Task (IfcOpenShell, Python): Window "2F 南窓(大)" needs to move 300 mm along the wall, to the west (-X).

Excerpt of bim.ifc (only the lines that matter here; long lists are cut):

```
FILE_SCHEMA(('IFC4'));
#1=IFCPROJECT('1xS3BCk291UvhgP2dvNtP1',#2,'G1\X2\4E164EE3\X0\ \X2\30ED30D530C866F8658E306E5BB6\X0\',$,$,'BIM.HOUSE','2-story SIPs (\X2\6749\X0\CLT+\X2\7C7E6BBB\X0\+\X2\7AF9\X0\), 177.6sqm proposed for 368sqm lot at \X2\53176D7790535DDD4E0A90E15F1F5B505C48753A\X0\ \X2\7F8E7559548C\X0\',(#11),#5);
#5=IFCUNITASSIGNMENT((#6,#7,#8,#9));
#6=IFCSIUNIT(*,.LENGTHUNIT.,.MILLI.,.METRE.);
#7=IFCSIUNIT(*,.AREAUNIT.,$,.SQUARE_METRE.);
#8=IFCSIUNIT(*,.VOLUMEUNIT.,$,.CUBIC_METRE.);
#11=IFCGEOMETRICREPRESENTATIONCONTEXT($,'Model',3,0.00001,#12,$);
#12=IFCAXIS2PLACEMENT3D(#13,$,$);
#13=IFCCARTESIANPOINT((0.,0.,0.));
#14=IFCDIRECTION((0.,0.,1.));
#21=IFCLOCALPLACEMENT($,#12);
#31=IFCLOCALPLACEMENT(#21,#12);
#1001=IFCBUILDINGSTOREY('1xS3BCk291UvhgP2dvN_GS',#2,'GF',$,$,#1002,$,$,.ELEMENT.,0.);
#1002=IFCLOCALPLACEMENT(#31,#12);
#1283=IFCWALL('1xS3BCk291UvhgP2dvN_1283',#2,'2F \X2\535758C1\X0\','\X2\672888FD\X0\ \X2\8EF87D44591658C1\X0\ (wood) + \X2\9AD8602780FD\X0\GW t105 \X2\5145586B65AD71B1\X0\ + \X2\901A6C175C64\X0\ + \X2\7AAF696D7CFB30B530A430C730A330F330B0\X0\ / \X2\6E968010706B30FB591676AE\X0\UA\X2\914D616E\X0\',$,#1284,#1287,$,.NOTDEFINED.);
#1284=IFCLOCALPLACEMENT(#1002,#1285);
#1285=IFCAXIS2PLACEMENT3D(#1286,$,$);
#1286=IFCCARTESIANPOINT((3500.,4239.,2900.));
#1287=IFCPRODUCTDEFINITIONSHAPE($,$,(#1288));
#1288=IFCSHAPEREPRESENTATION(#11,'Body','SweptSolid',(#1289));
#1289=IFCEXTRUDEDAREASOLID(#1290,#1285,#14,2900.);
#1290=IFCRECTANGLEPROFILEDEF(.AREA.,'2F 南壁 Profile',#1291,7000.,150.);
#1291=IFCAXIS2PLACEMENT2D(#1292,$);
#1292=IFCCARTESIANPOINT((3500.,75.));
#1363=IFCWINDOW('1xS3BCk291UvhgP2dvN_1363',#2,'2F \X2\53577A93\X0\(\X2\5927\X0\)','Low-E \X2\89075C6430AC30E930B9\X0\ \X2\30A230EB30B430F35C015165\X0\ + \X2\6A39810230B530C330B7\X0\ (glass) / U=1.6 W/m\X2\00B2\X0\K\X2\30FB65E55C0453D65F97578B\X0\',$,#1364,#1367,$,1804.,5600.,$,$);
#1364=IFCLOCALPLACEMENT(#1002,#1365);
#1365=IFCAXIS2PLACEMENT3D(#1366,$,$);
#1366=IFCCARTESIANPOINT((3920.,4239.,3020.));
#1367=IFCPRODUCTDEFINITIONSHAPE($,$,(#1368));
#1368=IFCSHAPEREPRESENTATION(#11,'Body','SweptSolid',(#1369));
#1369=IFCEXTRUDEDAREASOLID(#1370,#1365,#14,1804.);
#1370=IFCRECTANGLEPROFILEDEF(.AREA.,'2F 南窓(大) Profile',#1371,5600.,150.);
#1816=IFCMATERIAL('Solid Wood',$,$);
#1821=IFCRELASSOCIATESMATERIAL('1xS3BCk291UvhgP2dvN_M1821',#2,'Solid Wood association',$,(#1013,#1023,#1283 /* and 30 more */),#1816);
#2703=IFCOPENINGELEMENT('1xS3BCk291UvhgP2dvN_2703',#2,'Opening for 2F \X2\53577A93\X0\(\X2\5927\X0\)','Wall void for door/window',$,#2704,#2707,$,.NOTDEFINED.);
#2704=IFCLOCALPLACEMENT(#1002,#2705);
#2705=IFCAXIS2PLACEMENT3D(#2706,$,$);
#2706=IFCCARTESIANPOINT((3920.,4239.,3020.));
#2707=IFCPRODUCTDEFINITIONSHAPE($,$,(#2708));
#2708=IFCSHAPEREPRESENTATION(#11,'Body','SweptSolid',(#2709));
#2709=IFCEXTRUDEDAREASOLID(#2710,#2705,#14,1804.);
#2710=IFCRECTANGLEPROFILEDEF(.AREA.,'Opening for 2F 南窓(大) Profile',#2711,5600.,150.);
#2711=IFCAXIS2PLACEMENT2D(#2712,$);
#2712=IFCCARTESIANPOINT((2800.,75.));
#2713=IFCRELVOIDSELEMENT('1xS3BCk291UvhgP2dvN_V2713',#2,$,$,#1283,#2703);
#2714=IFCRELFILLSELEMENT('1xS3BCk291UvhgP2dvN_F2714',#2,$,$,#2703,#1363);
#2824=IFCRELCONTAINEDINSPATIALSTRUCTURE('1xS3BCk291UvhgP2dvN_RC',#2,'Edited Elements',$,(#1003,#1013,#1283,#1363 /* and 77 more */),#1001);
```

```python
import ifcopenshell
import ifcopenshell.api.geometry
import ifcopenshell.util.placement

model = ifcopenshell.open("bim.ifc")

window = model.by_guid("1xS3BCk291UvhgP2dvN_1363")
opening = window.FillsVoids[0].RelatingOpeningElement
wall = opening.VoidsElements[0].RelatingBuildingElement

wall_matrix = ifcopenshell.util.placement.get_local_placement(wall.ObjectPlacement)
shift = wall_matrix[:3, 0] * -300.0
before = ifcopenshell.util.placement.get_local_placement(window.ObjectPlacement)[:3, 3].copy()

# The window is not placed relative to its opening, so move both.
for product in (opening, window):
    matrix = ifcopenshell.util.placement.get_local_placement(product.ObjectPlacement)
    matrix[:3, 3] += shift
    ifcopenshell.api.geometry.edit_object_placement(model, product=product, matrix=matrix, is_si=False)

after = ifcopenshell.util.placement.get_local_placement(window.ObjectPlacement)[:3, 3]
print("window moved by", (after - before).round(3) + 0.0)

model.write("bim_updated.ifc")
```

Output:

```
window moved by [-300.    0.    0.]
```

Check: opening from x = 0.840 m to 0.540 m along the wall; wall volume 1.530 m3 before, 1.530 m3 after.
